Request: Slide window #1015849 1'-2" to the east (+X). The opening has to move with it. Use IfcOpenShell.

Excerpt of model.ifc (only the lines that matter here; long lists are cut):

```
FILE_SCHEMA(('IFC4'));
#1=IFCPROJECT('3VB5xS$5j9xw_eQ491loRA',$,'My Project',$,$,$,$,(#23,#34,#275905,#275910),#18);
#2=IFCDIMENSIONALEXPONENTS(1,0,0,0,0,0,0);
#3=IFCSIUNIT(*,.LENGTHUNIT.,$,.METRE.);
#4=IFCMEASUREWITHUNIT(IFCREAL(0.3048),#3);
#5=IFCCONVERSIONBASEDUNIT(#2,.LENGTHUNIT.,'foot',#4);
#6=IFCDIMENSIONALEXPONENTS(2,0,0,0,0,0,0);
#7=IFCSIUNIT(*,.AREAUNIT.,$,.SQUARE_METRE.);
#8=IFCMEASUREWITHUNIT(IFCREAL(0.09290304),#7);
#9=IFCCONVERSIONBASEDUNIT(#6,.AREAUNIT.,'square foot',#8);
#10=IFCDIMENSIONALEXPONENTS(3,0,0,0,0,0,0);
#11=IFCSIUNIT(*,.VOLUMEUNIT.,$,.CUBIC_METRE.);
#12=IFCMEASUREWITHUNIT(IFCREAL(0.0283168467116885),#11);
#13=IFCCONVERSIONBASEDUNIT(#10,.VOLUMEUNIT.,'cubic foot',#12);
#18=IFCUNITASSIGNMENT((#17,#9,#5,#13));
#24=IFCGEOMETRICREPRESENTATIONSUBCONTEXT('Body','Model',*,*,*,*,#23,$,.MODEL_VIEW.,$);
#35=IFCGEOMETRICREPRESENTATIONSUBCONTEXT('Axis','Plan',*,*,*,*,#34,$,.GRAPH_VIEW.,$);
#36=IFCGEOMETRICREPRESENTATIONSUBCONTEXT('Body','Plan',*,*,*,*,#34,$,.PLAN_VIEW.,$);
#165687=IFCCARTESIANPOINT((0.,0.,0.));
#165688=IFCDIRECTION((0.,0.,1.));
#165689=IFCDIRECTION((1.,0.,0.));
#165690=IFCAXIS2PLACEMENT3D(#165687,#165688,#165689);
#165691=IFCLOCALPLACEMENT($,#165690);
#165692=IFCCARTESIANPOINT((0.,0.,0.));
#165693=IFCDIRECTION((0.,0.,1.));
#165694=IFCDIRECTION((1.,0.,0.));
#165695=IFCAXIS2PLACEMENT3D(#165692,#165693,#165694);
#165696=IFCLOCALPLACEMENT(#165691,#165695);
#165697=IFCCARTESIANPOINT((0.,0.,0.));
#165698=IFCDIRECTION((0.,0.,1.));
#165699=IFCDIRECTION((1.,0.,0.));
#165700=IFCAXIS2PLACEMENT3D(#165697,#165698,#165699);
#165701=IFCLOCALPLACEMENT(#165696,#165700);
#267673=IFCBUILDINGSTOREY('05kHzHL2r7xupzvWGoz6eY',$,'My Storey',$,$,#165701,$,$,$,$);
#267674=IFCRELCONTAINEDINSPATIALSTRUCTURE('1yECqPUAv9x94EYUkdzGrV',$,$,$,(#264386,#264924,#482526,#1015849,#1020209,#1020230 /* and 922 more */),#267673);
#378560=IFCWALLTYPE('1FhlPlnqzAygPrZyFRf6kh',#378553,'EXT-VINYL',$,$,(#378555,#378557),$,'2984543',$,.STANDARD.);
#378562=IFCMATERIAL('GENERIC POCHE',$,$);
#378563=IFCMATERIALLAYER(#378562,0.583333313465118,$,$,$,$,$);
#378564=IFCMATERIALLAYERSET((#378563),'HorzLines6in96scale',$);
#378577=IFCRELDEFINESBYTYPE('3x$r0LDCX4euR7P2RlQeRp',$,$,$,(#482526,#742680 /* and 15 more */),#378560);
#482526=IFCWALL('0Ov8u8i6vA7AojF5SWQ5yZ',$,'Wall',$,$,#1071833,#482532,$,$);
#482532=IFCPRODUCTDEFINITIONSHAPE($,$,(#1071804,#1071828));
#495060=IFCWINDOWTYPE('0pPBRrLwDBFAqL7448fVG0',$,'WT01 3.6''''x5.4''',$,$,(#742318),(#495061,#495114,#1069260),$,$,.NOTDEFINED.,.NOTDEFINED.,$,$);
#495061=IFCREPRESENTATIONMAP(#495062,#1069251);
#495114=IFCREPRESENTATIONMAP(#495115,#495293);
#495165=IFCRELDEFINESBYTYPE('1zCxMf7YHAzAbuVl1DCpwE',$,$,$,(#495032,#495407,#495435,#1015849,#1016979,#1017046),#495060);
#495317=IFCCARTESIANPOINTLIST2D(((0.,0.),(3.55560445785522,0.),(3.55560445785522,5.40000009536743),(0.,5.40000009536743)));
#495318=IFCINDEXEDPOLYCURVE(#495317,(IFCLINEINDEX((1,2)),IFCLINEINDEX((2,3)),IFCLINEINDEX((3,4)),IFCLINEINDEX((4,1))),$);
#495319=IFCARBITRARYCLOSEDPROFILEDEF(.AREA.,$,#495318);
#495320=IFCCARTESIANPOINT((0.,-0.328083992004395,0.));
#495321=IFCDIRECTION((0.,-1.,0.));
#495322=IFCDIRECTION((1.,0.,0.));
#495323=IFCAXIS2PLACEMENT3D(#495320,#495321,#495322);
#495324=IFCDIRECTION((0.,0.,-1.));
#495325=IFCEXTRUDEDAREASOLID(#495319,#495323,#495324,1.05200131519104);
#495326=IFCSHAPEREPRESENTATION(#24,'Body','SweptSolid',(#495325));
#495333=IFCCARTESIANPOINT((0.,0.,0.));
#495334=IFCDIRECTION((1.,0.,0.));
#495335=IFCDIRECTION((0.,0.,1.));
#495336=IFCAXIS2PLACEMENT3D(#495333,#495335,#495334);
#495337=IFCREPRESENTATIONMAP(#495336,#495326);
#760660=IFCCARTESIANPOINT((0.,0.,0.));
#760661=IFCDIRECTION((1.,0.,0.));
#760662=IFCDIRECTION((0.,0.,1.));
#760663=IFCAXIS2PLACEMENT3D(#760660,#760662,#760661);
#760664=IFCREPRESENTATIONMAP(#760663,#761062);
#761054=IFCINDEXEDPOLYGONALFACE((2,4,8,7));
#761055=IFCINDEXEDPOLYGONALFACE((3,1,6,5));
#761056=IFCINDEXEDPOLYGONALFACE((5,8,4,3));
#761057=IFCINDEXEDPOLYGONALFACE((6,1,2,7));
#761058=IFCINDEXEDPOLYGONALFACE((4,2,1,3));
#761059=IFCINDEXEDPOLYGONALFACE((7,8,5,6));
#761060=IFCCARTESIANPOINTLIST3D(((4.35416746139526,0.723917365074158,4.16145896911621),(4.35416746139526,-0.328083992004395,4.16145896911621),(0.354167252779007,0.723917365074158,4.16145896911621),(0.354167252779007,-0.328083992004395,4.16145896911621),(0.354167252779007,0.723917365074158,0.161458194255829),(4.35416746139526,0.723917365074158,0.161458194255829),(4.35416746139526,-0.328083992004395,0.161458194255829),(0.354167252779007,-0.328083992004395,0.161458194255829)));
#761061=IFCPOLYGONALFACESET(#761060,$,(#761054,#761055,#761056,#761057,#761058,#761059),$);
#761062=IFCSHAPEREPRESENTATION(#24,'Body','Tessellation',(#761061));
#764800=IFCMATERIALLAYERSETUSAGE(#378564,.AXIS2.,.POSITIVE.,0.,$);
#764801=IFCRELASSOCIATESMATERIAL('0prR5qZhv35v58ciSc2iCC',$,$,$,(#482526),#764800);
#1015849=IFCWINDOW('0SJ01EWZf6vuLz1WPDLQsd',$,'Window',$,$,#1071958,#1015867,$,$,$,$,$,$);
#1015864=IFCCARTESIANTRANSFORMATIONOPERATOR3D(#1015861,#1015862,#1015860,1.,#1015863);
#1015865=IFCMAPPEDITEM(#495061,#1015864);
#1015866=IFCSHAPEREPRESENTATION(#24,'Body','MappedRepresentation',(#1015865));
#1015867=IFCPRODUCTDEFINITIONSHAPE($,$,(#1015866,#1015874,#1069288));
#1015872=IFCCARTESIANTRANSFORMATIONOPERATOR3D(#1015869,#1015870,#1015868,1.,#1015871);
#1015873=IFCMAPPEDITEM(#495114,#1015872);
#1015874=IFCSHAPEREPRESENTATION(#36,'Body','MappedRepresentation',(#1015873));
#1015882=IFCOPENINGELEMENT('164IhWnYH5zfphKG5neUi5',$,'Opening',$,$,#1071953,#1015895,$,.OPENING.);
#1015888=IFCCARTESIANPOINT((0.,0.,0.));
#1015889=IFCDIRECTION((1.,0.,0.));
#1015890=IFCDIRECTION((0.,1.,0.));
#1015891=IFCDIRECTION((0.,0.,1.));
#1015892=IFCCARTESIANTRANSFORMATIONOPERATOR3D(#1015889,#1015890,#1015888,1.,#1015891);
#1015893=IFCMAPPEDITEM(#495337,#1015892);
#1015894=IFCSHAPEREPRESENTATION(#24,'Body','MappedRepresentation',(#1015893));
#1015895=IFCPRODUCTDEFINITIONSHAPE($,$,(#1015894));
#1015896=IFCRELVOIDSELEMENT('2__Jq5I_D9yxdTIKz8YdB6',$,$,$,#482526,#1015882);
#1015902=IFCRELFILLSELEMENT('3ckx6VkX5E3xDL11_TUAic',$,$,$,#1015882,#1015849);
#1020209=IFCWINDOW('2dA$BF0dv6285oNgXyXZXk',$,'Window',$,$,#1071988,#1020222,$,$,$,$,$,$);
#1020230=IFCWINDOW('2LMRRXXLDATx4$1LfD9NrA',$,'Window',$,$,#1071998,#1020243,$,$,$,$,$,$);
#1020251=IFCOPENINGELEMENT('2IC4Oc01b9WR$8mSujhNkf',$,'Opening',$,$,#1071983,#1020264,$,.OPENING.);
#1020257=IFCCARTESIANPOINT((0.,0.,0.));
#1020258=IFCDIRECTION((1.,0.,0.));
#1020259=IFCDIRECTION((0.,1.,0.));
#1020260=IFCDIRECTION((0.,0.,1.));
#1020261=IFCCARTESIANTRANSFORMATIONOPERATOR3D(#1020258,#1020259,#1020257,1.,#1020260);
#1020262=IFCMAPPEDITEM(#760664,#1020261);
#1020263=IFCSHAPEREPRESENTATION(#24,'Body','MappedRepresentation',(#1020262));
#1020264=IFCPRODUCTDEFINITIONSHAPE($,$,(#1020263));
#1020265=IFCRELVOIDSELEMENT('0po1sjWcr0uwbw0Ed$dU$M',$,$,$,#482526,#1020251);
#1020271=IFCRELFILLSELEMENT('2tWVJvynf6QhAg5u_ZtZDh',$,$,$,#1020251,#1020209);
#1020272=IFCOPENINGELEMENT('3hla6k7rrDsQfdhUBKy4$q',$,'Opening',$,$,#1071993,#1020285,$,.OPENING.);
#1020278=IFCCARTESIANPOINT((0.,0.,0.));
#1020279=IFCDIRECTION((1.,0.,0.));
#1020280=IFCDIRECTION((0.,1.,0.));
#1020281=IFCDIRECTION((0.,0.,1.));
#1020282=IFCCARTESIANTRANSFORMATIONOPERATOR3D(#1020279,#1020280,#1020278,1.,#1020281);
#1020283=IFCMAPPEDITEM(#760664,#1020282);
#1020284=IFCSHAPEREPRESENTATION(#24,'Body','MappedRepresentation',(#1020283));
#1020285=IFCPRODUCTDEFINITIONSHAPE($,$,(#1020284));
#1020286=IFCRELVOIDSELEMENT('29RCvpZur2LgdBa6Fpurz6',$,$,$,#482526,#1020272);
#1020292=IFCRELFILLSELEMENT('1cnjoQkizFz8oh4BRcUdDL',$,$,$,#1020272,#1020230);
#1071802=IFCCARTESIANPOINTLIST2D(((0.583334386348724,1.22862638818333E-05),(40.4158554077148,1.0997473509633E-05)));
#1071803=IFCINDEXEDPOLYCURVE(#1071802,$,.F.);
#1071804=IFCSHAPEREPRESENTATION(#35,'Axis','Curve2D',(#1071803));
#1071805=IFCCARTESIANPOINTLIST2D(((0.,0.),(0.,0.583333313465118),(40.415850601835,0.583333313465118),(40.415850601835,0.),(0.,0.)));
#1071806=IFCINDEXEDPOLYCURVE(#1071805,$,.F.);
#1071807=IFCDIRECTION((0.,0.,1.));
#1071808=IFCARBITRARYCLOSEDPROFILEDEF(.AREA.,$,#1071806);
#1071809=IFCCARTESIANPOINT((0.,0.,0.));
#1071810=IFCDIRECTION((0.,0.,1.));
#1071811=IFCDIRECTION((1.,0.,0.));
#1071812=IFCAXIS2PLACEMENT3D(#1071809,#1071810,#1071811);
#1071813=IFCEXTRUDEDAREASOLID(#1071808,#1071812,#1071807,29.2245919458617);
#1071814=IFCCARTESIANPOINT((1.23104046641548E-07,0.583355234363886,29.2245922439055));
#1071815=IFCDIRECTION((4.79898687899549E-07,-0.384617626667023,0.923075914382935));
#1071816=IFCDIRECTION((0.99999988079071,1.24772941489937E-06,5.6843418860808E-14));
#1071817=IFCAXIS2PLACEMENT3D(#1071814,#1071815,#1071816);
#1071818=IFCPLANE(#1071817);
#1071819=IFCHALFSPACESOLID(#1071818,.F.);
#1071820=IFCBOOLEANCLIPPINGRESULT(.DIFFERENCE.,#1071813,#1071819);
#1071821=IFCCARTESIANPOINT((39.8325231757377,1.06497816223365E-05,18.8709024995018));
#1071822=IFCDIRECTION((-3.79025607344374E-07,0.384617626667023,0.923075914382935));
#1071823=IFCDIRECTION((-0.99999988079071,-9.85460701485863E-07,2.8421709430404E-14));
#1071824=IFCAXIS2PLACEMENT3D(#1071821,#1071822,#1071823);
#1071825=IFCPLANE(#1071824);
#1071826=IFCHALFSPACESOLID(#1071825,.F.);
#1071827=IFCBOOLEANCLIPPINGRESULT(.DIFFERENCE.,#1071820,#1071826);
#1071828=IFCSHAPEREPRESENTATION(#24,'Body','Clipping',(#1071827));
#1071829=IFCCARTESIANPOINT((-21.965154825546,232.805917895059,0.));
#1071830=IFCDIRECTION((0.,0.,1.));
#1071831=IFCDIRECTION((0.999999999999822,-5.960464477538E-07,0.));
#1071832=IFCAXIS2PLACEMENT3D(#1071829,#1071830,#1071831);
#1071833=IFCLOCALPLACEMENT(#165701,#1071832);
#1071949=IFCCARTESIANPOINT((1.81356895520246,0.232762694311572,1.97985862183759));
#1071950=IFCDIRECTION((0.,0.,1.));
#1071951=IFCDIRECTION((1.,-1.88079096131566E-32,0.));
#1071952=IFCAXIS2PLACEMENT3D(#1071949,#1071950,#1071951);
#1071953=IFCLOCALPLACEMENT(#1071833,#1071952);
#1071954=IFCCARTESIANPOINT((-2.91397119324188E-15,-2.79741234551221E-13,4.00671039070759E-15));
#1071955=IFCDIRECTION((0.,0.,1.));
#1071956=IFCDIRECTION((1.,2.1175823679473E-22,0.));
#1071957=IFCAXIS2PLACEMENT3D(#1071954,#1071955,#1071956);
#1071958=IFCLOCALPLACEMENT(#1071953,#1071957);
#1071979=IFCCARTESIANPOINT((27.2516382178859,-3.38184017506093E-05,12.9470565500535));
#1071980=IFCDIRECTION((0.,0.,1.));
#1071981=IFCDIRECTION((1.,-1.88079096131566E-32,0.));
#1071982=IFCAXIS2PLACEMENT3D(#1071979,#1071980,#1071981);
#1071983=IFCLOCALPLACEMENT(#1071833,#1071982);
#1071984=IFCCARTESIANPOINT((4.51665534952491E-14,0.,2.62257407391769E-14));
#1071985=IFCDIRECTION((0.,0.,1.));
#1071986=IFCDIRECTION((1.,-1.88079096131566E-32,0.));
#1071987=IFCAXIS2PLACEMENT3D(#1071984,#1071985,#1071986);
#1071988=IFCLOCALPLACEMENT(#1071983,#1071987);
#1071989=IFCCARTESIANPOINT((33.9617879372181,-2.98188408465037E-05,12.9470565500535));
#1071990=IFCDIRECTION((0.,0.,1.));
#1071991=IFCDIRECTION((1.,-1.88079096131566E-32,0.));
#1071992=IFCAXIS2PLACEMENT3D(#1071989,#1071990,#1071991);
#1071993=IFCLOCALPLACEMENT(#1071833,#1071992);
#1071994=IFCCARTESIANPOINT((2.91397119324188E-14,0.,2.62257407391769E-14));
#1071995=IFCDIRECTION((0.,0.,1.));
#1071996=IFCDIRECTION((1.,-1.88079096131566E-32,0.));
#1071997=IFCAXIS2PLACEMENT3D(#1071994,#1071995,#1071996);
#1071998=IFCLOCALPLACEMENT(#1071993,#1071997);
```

```python
import ifcopenshell
import ifcopenshell.api.geometry
import ifcopenshell.util.placement
import ifcopenshell.util.unit

model = ifcopenshell.open("model.ifc")
unit_scale = ifcopenshell.util.unit.calculate_unit_scale(model)

window = model.by_guid("0SJ01EWZf6vuLz1WPDLQsd")
opening = window.FillsVoids[0].RelatingOpeningElement
wall = opening.VoidsElements[0].RelatingBuildingElement

wall_matrix = ifcopenshell.util.placement.get_local_placement(wall.ObjectPlacement)
shift = wall_matrix[:3, 0] * 14 * 0.0254 / unit_scale
before = ifcopenshell.util.placement.get_local_placement(window.ObjectPlacement)[:3, 3].copy()

# The window is placed relative to its opening, so it follows when the opening moves.
matrix = ifcopenshell.util.placement.get_local_placement(opening.ObjectPlacement)
matrix[:3, 3] += shift
ifcopenshell.api.geometry.edit_object_placement(
    model, product=opening, matrix=matrix, is_si=False, should_transform_children=True
)

after = ifcopenshell.util.placement.get_local_placement(window.ObjectPlacement)[:3, 3]
print("window moved by", (after - before).round(3) + 0.0)

model.write("model_v2.ifc")
```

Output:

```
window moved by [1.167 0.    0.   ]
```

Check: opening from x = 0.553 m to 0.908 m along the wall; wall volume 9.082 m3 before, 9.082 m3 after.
